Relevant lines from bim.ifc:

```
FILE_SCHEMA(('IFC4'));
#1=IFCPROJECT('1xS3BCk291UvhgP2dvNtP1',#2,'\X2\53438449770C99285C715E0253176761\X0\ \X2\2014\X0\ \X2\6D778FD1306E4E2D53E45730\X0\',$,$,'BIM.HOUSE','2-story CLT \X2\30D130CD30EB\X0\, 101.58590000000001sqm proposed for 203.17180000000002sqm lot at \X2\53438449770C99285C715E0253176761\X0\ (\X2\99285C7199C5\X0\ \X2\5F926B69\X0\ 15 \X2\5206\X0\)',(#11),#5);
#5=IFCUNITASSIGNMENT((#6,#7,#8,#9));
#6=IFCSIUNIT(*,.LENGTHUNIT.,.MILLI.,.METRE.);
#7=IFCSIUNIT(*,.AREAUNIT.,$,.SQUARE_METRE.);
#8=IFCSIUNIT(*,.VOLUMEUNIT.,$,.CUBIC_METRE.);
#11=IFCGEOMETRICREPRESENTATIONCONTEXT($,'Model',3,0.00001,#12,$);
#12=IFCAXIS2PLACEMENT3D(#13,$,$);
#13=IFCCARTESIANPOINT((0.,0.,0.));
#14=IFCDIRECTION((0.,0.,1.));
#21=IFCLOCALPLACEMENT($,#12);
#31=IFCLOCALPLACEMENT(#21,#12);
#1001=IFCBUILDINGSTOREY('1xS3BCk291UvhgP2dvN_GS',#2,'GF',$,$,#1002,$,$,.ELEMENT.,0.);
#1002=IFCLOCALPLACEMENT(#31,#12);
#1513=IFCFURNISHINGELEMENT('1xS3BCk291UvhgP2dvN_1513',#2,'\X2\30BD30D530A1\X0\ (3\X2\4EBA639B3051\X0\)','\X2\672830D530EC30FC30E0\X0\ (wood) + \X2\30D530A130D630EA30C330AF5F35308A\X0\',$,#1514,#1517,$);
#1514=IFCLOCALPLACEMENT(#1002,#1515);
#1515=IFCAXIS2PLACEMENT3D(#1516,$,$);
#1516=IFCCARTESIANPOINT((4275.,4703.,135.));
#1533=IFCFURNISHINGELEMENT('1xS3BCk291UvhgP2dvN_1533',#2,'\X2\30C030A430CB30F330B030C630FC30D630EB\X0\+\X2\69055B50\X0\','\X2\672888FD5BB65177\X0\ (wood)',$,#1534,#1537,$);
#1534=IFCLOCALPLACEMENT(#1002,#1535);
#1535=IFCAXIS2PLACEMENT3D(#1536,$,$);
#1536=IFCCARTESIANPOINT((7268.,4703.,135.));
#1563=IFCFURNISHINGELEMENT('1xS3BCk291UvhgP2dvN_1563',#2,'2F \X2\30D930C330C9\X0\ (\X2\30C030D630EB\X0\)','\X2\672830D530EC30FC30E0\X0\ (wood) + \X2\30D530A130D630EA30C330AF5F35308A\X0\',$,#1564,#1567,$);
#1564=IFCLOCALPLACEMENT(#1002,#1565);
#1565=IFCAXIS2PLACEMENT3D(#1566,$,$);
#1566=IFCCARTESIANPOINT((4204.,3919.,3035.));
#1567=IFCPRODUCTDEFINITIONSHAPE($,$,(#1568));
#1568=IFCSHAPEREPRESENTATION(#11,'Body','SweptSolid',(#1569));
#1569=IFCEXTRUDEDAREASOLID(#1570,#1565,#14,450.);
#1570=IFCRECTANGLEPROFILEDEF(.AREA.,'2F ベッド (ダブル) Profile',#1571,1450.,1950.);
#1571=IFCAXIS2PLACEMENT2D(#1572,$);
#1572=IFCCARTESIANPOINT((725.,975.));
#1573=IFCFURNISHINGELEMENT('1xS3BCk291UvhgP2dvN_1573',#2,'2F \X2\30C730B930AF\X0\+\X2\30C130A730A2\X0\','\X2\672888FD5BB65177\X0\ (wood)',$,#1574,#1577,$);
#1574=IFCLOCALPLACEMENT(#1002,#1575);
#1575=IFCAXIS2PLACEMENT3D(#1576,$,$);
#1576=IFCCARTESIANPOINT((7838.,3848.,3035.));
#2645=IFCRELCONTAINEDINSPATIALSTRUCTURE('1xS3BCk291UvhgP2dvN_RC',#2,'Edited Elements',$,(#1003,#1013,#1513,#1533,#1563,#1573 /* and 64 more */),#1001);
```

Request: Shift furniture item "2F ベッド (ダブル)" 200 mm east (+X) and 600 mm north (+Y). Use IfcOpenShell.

```python
import ifcopenshell
import ifcopenshell.api.geometry
import ifcopenshell.util.placement
import ifcopenshell.util.unit

model = ifcopenshell.open("bim.ifc")
unit_scale = ifcopenshell.util.unit.calculate_unit_scale(model)

item = model.by_guid("1xS3BCk291UvhgP2dvN_1563")
matrix = ifcopenshell.util.placement.get_local_placement(item.ObjectPlacement)
matrix[0, 3] += 0.2 / unit_scale
matrix[1, 3] += 0.6 / unit_scale
ifcopenshell.api.geometry.edit_object_placement(model, product=item, matrix=matrix, is_si=False)

print(ifcopenshell.util.placement.get_local_placement(item.ObjectPlacement).round(3) + 0.0)

model.write("bim_updated.ifc")
```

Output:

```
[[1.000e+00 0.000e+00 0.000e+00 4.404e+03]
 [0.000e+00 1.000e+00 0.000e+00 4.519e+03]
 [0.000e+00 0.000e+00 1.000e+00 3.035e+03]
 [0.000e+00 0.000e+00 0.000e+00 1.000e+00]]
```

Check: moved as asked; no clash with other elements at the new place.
